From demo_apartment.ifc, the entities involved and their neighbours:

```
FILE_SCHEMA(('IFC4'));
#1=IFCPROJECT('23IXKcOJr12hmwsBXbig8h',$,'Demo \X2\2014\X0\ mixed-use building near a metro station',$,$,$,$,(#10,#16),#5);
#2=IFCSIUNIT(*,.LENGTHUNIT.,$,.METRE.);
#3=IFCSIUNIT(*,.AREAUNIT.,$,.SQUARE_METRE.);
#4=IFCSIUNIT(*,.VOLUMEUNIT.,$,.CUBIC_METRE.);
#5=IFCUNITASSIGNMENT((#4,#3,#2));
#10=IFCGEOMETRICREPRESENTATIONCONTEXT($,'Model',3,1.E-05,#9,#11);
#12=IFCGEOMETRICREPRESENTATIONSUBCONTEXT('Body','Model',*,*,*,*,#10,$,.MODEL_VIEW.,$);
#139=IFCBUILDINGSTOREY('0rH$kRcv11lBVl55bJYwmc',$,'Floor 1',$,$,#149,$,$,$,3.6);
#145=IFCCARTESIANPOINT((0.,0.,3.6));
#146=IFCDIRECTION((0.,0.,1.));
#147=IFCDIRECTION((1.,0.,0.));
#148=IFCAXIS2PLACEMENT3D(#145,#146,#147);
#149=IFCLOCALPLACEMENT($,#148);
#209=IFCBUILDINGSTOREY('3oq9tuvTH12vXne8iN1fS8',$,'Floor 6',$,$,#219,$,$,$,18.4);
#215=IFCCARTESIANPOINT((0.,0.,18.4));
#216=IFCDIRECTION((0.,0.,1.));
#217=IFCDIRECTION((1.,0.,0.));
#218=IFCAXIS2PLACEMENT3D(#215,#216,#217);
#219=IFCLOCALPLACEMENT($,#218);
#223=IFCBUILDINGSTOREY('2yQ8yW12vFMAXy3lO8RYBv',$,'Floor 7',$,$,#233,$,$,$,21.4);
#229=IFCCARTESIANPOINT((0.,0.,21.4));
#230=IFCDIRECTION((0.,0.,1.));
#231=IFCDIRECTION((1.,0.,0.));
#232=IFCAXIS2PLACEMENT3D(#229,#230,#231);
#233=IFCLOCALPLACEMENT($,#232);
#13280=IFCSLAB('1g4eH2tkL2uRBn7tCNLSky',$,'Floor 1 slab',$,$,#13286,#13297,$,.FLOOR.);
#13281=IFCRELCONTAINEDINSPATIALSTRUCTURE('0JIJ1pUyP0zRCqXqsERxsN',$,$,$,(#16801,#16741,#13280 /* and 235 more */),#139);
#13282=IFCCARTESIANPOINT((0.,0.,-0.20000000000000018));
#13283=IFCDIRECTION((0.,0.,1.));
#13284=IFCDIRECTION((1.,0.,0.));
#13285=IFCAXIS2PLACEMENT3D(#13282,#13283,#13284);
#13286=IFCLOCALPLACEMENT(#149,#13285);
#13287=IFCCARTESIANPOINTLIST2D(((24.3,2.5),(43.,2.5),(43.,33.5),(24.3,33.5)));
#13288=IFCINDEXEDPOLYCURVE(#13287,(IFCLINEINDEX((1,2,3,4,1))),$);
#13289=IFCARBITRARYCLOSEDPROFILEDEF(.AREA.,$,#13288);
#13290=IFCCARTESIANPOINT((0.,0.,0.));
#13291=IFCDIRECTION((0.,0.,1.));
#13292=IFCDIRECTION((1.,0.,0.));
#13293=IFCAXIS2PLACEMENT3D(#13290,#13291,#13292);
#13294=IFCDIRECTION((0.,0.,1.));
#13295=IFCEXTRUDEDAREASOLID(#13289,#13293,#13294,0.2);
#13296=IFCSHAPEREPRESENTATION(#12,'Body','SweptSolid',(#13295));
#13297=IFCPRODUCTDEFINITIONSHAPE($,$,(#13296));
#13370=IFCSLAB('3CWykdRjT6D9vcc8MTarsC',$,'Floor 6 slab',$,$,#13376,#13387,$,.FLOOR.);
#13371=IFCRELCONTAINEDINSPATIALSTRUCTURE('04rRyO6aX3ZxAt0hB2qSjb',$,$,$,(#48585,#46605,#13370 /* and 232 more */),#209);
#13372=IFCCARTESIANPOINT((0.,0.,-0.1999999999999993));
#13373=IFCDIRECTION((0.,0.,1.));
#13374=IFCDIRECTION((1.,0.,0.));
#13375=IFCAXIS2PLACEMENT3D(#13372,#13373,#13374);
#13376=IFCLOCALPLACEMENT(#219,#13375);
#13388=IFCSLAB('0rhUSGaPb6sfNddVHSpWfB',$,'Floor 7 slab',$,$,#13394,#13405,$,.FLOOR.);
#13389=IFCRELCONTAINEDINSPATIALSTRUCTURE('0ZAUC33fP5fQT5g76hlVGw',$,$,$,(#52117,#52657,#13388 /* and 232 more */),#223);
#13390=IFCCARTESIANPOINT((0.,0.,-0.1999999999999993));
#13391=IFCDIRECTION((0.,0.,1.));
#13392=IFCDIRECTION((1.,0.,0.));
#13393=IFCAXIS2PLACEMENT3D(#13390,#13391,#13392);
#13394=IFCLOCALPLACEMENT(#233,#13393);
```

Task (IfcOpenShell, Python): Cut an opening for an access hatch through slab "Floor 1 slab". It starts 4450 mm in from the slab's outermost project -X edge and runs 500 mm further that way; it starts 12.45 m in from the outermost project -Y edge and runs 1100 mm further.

```python
import numpy as np
import ifcopenshell
import ifcopenshell.api.feature
import ifcopenshell.api.geometry
import ifcopenshell.api.root
import ifcopenshell.geom
import ifcopenshell.util.placement
import ifcopenshell.util.representation
import ifcopenshell.util.shape
import ifcopenshell.util.unit

model = ifcopenshell.open("demo_apartment.ifc")
unit_scale = ifcopenshell.util.unit.calculate_unit_scale(model)
settings = ifcopenshell.geom.settings()


def volume(element):
    """Net volume in cubic metres, openings subtracted."""
    shape = ifcopenshell.geom.create_shape(settings, element)
    return ifcopenshell.util.shape.get_volume(shape.geometry)


slab = model.by_id(13280)
before = volume(slab)

# Extent in the slab's own axes, in metres. The edges named are its -X and -Y sides.
slab_shape = ifcopenshell.geom.create_shape(settings, slab)
vertices = ifcopenshell.util.shape.get_vertices(slab_shape.geometry)
x_min, y_min, bottom = vertices.min(axis=0)
top = vertices[:, 2].max()

opening = ifcopenshell.api.root.create_entity(model, ifc_class="IfcOpeningElement", name="Access hatch opening", predefined_type="OPENING")
context = ifcopenshell.util.representation.get_context(model, "Model", "Body", "MODEL_VIEW")
width, depth = 0.5, 1.1
outline = [(0.0, 0.0), (width, 0.0), (width, depth), (0.0, depth), (0.0, 0.0)]
# Overshoot both faces by 50 mm so the cut is clean.
shape = ifcopenshell.api.geometry.add_slab_representation(
    model, context=context, depth=top - bottom + 0.1, polyline=outline
)
ifcopenshell.api.geometry.assign_representation(model, product=opening, representation=shape)

matrix = ifcopenshell.util.placement.get_local_placement(slab.ObjectPlacement)
matrix[:, 3] = matrix @ np.append(np.array([x_min + 4.45, y_min + 12.45, bottom - 0.05]) / unit_scale, 1.0)
ifcopenshell.api.geometry.edit_object_placement(model, product=opening, matrix=matrix, is_si=False)
ifcopenshell.api.feature.add_feature(model, feature=opening, element=slab)

after = volume(slab)

print(f"slab volume {before:.3f} -> {after:.3f} m3")

model.write("demo_apartment_rev.ifc")
```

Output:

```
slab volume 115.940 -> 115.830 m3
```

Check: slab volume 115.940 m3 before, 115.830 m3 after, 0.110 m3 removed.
